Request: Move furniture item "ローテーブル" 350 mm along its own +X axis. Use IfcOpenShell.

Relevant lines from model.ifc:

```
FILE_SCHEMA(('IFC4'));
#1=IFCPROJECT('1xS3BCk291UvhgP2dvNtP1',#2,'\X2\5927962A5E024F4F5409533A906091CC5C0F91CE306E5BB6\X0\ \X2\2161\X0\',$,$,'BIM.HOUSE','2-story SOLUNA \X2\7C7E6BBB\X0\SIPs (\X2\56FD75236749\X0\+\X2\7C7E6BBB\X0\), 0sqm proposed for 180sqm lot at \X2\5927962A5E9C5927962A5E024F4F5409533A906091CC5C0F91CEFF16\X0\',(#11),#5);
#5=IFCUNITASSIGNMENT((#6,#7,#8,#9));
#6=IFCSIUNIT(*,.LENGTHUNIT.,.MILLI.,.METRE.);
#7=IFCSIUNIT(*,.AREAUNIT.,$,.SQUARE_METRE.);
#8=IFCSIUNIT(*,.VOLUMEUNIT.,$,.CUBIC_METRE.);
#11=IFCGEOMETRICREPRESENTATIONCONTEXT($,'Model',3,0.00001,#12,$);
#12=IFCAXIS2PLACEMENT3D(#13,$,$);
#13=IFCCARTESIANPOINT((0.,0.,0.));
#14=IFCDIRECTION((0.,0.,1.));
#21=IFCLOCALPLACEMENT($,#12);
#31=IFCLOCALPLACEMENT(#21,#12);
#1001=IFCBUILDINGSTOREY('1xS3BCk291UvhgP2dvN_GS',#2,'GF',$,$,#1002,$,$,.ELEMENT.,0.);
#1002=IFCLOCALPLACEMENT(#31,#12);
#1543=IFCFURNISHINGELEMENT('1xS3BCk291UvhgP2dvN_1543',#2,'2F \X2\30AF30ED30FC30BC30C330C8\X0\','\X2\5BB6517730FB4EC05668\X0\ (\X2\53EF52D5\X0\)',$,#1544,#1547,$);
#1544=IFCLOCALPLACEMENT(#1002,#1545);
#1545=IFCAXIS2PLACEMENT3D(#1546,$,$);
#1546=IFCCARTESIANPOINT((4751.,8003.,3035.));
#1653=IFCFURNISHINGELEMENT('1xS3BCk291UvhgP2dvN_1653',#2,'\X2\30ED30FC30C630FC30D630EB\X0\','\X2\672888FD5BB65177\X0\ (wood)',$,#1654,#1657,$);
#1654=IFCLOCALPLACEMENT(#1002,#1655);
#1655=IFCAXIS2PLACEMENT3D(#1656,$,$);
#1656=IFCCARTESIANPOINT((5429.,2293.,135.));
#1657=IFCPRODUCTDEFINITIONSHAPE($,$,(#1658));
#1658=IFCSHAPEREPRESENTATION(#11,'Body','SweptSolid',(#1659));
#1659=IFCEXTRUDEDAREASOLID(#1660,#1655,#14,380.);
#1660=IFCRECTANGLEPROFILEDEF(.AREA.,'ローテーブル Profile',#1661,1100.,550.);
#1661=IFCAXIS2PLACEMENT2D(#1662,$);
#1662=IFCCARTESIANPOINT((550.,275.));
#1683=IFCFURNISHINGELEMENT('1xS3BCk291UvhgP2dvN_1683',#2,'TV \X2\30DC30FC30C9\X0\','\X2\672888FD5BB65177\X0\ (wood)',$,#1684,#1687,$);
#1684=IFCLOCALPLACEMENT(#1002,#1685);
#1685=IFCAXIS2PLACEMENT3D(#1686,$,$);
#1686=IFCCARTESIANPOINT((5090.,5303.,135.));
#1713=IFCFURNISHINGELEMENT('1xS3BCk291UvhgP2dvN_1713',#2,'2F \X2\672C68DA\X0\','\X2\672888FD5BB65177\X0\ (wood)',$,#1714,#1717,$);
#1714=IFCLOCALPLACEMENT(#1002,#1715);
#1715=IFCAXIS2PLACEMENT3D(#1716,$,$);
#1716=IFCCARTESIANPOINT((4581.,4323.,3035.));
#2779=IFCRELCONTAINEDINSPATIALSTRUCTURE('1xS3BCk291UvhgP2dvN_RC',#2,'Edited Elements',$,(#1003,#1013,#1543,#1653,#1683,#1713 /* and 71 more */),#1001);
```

```python
import ifcopenshell
import ifcopenshell.api.geometry
import ifcopenshell.util.placement
import ifcopenshell.util.unit

model = ifcopenshell.open("model.ifc")
unit_scale = ifcopenshell.util.unit.calculate_unit_scale(model)

item = model.by_guid("1xS3BCk291UvhgP2dvN_1653")
matrix = ifcopenshell.util.placement.get_local_placement(item.ObjectPlacement)
matrix[:3, 3] += matrix[:3, 0] * 0.35 / unit_scale
ifcopenshell.api.geometry.edit_object_placement(model, product=item, matrix=matrix, is_si=False)

print(ifcopenshell.util.placement.get_local_placement(item.ObjectPlacement).round(3) + 0.0)

model.write("model_v2.ifc")
```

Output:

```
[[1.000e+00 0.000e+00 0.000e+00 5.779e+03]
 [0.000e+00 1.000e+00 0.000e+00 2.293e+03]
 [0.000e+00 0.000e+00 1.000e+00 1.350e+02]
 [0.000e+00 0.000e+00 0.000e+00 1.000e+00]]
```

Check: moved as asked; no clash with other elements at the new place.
